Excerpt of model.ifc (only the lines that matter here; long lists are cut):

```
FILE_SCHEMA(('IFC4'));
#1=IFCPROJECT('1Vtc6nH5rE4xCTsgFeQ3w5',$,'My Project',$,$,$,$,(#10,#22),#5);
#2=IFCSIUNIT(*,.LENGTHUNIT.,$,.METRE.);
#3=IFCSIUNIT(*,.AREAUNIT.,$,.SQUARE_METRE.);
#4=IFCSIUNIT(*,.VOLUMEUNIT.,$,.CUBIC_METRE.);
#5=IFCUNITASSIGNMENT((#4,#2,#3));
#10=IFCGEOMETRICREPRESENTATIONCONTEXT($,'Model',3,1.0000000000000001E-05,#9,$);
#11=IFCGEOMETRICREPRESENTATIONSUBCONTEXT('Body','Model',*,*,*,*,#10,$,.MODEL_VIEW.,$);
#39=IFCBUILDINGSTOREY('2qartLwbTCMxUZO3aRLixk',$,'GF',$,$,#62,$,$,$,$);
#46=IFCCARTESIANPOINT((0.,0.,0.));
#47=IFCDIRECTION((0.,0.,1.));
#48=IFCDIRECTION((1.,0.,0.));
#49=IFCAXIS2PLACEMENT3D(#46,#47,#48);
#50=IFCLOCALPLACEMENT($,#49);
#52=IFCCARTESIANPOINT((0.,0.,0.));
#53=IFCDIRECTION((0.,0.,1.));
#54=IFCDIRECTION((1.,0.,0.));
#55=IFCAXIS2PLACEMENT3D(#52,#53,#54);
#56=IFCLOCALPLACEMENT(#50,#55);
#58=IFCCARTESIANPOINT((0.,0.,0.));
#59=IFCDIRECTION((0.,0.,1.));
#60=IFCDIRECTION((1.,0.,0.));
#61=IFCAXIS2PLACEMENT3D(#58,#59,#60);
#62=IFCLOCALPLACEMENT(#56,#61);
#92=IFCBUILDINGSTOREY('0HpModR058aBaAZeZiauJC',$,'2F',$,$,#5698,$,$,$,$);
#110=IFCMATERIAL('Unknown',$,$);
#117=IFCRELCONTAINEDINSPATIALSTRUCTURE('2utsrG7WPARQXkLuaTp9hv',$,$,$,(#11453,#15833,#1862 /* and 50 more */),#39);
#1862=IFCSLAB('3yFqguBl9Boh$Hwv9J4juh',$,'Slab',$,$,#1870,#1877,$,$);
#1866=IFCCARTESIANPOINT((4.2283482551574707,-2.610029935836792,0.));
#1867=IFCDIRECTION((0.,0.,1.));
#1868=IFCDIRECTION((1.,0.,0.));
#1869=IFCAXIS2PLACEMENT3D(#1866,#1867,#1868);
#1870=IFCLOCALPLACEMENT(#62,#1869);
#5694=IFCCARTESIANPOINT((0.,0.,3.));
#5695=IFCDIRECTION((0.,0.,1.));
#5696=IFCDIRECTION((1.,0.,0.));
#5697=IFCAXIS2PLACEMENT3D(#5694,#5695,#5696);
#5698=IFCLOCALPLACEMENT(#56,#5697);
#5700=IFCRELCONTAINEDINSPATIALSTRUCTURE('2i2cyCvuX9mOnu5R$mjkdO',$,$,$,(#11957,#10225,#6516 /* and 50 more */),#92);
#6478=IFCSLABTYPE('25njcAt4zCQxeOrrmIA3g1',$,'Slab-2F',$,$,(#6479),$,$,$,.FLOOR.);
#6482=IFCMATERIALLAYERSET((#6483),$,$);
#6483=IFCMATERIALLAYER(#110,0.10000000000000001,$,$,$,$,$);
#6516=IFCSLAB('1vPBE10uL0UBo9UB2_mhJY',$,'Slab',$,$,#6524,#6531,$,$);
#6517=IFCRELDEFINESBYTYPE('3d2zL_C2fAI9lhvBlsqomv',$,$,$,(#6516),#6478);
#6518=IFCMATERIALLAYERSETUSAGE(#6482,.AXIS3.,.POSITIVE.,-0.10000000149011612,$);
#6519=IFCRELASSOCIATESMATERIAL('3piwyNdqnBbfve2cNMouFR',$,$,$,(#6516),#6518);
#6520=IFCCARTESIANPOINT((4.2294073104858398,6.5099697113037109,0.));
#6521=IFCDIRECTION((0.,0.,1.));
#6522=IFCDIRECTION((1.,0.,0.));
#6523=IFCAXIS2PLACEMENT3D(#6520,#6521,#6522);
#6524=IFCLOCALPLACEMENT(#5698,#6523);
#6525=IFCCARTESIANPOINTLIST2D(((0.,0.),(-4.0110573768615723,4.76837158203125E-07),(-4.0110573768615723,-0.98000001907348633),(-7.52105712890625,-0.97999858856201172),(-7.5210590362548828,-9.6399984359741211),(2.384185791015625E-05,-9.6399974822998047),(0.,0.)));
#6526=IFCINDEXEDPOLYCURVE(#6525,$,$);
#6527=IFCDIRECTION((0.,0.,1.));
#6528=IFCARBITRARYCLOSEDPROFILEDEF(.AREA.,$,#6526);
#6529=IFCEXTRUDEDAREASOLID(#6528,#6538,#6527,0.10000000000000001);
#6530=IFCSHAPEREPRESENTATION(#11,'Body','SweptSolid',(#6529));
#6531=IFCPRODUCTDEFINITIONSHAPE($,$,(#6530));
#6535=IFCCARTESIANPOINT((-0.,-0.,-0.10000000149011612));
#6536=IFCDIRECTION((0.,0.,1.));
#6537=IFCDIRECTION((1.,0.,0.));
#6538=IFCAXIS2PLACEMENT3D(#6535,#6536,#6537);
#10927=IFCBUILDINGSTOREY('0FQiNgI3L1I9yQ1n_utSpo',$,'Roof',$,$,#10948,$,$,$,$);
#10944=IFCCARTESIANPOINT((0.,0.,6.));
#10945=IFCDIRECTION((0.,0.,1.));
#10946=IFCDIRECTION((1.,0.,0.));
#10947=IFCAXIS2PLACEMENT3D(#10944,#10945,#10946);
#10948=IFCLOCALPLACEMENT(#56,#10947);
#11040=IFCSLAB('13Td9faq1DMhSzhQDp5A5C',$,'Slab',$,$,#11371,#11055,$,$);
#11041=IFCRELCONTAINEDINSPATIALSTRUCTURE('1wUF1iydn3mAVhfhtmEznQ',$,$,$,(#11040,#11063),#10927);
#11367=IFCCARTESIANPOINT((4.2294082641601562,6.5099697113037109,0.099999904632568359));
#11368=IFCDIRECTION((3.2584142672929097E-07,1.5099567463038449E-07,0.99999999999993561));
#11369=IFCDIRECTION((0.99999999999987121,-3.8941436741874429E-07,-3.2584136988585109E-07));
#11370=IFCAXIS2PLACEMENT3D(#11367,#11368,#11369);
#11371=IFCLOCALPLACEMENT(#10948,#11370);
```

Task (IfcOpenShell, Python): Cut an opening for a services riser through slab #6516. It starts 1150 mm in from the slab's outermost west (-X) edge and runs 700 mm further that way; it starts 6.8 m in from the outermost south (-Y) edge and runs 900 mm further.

```python
import numpy as np
import ifcopenshell
import ifcopenshell.api.feature
import ifcopenshell.api.geometry
import ifcopenshell.api.root
import ifcopenshell.geom
import ifcopenshell.util.placement
import ifcopenshell.util.representation
import ifcopenshell.util.shape
import ifcopenshell.util.unit

model = ifcopenshell.open("model.ifc")
unit_scale = ifcopenshell.util.unit.calculate_unit_scale(model)
settings = ifcopenshell.geom.settings()


def volume(element):
    """Net volume in cubic metres, openings subtracted."""
    shape = ifcopenshell.geom.create_shape(settings, element)
    return ifcopenshell.util.shape.get_volume(shape.geometry)


slab = model.by_guid("1vPBE10uL0UBo9UB2_mhJY")
before = volume(slab)

# Extent in the slab's own axes, in metres. The edges named are its -X and -Y sides.
slab_shape = ifcopenshell.geom.create_shape(settings, slab)
vertices = ifcopenshell.util.shape.get_vertices(slab_shape.geometry)
x_min, y_min, bottom = vertices.min(axis=0)
top = vertices[:, 2].max()

opening = ifcopenshell.api.root.create_entity(model, ifc_class="IfcOpeningElement", name="Services riser opening", predefined_type="OPENING")
context = ifcopenshell.util.representation.get_context(model, "Model", "Body", "MODEL_VIEW")
width, depth = 0.7, 0.9
outline = [(0.0, 0.0), (width, 0.0), (width, depth), (0.0, depth), (0.0, 0.0)]
# Overshoot both faces by 50 mm so the cut is clean.
shape = ifcopenshell.api.geometry.add_slab_representation(
    model, context=context, depth=top - bottom + 0.1, polyline=outline
)
ifcopenshell.api.geometry.assign_representation(model, product=opening, representation=shape)

matrix = ifcopenshell.util.placement.get_local_placement(slab.ObjectPlacement)
matrix[:, 3] = matrix @ np.append(np.array([x_min + 1.15, y_min + 6.8, bottom - 0.05]) / unit_scale, 1.0)
ifcopenshell.api.geometry.edit_object_placement(model, product=opening, matrix=matrix, is_si=False)
ifcopenshell.api.feature.add_feature(model, feature=opening, element=slab)

after = volume(slab)

print(f"slab volume {before:.3f} -> {after:.3f} m3")

model.write("model_edited.ifc")
```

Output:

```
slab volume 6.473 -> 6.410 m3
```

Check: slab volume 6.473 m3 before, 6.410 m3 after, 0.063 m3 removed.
